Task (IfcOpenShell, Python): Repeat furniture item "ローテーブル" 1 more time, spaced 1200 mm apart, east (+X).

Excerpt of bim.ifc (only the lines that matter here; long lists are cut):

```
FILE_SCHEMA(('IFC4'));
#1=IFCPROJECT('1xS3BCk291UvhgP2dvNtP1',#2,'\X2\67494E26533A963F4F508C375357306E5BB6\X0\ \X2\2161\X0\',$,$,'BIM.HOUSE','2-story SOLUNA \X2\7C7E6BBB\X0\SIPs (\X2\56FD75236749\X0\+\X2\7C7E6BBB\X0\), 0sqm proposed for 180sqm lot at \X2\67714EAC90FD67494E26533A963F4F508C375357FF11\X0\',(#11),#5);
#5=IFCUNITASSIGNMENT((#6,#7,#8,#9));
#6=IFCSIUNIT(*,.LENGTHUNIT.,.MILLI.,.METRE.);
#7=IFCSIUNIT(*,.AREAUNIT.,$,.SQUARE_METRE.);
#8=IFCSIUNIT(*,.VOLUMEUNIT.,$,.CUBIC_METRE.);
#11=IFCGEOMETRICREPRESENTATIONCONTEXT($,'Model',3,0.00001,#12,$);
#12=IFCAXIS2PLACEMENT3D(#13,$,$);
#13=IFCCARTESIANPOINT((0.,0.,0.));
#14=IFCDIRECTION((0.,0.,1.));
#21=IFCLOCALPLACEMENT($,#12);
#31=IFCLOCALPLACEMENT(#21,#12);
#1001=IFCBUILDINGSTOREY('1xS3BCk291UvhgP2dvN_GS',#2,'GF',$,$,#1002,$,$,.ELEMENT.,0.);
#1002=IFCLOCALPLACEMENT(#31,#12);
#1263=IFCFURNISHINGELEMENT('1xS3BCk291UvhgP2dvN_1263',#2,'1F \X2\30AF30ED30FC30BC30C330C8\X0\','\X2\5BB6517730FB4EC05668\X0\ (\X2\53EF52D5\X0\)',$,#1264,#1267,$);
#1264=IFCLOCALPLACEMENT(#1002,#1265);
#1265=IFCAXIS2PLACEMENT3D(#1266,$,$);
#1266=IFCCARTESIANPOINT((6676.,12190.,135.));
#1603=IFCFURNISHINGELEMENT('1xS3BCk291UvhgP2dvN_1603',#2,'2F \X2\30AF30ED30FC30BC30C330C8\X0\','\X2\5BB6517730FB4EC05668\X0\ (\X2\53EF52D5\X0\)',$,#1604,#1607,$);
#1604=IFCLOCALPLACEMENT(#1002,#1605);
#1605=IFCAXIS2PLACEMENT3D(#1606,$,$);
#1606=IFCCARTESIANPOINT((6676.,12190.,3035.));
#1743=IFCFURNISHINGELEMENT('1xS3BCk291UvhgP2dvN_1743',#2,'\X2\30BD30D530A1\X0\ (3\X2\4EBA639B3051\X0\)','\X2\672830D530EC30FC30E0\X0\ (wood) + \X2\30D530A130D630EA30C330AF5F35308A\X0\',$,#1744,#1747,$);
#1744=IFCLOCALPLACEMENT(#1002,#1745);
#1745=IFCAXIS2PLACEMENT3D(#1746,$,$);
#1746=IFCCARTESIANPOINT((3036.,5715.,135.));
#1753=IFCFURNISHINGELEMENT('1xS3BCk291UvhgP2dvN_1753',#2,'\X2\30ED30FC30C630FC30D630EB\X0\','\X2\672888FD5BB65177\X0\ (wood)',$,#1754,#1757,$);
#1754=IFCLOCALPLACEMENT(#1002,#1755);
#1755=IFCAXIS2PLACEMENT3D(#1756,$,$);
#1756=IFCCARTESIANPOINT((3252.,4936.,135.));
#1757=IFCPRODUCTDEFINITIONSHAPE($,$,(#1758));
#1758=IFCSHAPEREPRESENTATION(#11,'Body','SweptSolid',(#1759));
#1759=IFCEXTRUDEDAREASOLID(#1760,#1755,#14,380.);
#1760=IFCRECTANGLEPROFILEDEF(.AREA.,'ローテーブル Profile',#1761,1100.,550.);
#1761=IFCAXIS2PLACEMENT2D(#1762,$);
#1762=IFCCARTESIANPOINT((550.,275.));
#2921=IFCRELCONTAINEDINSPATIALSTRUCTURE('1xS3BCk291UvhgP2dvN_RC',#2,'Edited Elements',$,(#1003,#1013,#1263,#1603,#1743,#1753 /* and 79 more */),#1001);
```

```python
import numpy as np
import ifcopenshell
import ifcopenshell.api.geometry
import ifcopenshell.api.root
import ifcopenshell.util.element
import ifcopenshell.util.placement

model = ifcopenshell.open("bim.ifc")


def reuse_history(source, copy):
    """copy_class also copies each property set's owner history, people and application; keep the originals."""
    for rel in copy.IsDefinedBy:
        if rel.is_a("IfcRelDefinesByProperties") and (history := rel.RelatingPropertyDefinition.OwnerHistory):
            rel.RelatingPropertyDefinition.OwnerHistory = source.OwnerHistory
            ifcopenshell.util.element.remove_deep2(model, history)


source = model.by_guid("1xS3BCk291UvhgP2dvN_1753")
base = ifcopenshell.util.placement.get_local_placement(source.ObjectPlacement)
step = np.array([1.0, 0.0, 0.0]) * 1200.0

for i in range(1, 2):
    copy = ifcopenshell.api.root.copy_class(model, product=source)
    copy.Representation = ifcopenshell.util.element.copy_deep(
        model, source.Representation, exclude=["IfcGeometricRepresentationContext", "IfcRepresentationMap"]
    )
    reuse_history(source, copy)
    matrix = base.copy()
    matrix[:3, 3] += i * step
    print("added at", matrix[:3, 3].round(3) + 0.0)
    ifcopenshell.api.geometry.edit_object_placement(model, product=copy, matrix=matrix, is_si=False)

model.write("bim_updated.ifc")
```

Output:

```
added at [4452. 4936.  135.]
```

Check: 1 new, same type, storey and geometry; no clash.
